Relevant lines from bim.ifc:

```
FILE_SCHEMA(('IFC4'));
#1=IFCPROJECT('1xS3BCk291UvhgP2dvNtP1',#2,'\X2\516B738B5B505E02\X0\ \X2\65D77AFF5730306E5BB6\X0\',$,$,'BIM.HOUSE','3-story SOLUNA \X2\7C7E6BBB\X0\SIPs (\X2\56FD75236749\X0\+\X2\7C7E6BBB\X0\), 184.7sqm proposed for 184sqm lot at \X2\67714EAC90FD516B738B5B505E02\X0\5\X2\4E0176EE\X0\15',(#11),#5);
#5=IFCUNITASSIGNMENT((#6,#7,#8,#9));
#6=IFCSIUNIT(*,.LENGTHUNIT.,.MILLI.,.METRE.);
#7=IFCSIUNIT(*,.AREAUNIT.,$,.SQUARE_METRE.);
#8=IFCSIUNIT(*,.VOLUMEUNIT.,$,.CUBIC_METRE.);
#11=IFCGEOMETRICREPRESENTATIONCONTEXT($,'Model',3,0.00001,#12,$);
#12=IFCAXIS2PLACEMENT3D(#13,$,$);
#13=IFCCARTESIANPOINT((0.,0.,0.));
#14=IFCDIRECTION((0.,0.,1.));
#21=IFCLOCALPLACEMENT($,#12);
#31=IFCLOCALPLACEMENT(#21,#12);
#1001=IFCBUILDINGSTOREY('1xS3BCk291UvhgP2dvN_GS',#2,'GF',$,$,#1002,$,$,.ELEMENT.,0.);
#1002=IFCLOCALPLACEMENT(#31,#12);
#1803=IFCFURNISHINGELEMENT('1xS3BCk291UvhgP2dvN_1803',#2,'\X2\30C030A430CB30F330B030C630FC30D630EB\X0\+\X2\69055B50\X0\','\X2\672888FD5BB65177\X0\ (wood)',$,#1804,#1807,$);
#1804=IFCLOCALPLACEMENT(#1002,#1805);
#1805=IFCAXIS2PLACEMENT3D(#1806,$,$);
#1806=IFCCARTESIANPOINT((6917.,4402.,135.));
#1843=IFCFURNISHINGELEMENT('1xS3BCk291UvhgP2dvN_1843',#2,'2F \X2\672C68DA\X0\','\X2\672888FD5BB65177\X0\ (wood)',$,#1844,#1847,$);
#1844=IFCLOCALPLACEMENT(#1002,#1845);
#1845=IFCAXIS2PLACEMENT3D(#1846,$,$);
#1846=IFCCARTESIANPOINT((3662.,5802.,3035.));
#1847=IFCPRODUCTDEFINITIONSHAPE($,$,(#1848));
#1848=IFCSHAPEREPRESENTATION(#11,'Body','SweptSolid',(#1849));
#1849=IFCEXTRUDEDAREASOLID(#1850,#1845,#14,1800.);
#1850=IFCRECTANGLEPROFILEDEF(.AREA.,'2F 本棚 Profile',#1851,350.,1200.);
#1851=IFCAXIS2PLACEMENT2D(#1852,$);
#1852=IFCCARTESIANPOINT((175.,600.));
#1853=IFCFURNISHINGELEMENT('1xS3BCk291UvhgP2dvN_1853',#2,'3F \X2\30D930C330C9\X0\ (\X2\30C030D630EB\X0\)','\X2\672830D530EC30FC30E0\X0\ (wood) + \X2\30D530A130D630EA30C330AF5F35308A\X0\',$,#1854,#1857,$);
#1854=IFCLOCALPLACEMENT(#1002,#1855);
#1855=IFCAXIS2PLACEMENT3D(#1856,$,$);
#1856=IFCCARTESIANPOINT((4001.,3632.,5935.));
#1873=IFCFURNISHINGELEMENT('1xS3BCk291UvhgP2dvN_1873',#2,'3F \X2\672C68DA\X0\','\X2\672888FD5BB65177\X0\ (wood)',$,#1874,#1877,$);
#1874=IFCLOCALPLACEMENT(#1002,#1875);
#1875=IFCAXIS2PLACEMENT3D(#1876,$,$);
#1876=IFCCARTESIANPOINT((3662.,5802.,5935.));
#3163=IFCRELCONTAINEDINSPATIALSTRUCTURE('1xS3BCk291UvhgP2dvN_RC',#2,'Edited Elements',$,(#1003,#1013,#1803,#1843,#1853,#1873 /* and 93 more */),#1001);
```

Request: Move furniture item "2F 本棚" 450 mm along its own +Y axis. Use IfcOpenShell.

```python
import ifcopenshell
import ifcopenshell.api.geometry
import ifcopenshell.util.placement

model = ifcopenshell.open("bim.ifc")

item = model.by_guid("1xS3BCk291UvhgP2dvN_1843")
matrix = ifcopenshell.util.placement.get_local_placement(item.ObjectPlacement)
matrix[:3, 3] += matrix[:3, 1] * 450.0
ifcopenshell.api.geometry.edit_object_placement(model, product=item, matrix=matrix, is_si=False)

print(ifcopenshell.util.placement.get_local_placement(item.ObjectPlacement).round(3) + 0.0)

model.write("bim_v2.ifc")
```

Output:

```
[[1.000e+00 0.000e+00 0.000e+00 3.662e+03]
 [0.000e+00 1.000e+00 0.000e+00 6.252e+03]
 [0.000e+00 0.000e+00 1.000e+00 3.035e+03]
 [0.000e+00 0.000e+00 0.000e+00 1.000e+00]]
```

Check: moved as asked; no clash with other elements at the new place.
